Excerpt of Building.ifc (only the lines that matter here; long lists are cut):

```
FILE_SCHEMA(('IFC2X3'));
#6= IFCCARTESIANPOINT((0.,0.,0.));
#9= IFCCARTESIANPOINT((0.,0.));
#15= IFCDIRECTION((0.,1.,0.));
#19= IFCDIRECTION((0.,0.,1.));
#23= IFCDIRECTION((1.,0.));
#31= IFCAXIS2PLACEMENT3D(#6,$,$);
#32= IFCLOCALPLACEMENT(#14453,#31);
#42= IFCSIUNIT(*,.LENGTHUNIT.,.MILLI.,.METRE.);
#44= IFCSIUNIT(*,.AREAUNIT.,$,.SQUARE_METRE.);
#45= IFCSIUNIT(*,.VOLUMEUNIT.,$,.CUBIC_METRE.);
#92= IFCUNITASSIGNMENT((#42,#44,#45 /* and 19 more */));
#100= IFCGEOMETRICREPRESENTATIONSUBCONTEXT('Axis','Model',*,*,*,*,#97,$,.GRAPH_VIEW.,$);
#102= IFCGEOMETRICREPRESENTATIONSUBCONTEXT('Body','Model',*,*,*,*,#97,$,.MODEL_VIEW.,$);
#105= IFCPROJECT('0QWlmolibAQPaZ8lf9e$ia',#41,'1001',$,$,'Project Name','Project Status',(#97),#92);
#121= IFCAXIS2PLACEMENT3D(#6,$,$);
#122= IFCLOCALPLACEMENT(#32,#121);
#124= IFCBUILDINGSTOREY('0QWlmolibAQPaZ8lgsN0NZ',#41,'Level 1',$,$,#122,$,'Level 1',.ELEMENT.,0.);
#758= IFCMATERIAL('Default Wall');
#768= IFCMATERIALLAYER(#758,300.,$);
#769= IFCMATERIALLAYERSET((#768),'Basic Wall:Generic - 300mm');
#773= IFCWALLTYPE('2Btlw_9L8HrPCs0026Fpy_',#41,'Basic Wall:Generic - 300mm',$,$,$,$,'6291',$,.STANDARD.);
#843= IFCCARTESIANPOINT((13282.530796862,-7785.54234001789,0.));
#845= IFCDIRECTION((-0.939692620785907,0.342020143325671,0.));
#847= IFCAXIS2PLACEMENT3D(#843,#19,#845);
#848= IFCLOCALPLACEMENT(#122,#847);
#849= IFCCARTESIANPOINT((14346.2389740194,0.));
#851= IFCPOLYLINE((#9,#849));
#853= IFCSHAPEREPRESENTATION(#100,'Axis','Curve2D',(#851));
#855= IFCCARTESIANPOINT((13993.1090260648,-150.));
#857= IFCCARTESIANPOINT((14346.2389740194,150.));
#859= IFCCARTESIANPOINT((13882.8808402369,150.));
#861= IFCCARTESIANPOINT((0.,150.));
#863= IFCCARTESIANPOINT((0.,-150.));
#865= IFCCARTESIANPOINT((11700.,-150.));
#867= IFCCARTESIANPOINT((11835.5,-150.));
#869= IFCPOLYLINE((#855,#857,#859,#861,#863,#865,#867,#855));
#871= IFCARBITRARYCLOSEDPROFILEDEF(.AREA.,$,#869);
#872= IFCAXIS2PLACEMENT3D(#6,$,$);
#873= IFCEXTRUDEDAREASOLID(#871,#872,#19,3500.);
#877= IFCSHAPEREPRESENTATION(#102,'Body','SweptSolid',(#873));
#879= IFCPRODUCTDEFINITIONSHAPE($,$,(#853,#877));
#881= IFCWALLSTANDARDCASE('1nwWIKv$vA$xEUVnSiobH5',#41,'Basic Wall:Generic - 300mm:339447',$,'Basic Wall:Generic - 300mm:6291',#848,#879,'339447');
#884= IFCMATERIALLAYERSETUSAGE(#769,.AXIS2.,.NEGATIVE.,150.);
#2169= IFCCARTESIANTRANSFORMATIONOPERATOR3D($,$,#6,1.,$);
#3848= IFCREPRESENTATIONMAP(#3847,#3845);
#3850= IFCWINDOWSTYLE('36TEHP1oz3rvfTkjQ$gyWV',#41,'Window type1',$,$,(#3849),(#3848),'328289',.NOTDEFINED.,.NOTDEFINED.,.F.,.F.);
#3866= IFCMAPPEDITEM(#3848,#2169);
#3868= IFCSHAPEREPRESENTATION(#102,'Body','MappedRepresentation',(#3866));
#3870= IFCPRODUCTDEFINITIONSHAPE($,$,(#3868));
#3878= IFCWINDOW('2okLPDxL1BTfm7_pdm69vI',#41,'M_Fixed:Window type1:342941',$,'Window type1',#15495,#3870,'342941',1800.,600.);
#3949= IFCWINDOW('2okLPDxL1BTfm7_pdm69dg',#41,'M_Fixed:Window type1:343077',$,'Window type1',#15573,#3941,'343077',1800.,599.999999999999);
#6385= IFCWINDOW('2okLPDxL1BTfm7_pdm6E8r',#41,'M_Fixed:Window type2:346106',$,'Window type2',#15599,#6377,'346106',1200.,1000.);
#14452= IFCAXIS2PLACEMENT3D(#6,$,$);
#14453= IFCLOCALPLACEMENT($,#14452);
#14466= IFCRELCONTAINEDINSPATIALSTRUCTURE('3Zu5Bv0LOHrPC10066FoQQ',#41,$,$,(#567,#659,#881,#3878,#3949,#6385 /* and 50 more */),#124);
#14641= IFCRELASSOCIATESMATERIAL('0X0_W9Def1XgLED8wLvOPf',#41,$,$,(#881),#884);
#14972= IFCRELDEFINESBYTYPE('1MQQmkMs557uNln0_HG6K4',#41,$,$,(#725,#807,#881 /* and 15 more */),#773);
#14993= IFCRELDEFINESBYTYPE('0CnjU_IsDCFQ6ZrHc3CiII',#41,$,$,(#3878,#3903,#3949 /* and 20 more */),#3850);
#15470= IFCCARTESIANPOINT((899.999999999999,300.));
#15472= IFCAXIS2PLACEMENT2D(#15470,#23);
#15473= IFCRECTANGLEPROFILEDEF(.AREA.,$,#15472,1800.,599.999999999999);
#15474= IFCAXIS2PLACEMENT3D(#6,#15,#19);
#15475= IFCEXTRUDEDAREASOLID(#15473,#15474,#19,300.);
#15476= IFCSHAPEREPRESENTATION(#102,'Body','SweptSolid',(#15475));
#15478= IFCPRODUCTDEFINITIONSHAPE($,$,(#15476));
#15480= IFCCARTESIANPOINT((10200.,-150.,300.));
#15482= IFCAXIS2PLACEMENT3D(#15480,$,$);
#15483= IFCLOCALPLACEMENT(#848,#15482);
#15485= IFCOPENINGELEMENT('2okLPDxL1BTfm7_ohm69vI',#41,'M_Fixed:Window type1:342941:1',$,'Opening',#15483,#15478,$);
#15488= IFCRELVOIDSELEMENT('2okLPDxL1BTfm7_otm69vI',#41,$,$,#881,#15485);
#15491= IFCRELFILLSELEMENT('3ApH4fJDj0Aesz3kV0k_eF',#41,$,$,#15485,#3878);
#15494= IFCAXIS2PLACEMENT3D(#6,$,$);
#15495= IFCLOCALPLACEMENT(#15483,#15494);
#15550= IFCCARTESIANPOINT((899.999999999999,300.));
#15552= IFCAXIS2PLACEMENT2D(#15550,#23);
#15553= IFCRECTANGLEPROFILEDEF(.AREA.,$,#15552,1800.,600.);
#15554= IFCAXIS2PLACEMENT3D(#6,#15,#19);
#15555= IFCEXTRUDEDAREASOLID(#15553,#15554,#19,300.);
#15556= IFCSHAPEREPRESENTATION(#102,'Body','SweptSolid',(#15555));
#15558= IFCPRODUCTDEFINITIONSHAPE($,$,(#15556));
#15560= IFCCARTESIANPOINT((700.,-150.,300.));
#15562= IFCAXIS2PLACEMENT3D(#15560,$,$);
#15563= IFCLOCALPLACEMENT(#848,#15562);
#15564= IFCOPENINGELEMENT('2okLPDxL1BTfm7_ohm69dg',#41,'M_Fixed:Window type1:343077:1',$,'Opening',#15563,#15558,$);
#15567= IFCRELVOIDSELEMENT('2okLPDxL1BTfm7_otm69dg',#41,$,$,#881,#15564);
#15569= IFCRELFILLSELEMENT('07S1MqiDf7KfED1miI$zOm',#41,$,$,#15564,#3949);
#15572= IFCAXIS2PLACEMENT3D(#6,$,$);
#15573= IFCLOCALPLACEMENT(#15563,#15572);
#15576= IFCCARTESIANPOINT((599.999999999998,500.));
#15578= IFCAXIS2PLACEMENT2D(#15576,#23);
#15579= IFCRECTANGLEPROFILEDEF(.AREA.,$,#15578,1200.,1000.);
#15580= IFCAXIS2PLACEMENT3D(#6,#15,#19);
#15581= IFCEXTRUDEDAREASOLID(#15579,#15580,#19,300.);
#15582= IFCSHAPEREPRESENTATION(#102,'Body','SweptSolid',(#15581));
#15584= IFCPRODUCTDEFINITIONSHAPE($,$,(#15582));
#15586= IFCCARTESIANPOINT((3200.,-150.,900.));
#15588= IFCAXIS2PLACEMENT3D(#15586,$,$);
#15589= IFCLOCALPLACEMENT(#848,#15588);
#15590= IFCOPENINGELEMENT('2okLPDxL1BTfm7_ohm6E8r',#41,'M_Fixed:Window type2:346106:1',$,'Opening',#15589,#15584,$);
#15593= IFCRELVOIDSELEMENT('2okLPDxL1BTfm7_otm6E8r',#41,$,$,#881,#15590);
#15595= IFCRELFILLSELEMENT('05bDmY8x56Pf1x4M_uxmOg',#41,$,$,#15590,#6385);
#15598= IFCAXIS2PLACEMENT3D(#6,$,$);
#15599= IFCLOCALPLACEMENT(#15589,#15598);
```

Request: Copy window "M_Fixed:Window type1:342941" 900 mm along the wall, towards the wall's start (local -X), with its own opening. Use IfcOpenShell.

```python
import ifcopenshell
import ifcopenshell.api.feature
import ifcopenshell.api.geometry
import ifcopenshell.api.root
import ifcopenshell.geom
import ifcopenshell.util.element
import ifcopenshell.util.placement
import ifcopenshell.util.shape
import ifcopenshell.util.unit

model = ifcopenshell.open("Building.ifc")
unit_scale = ifcopenshell.util.unit.calculate_unit_scale(model)
settings = ifcopenshell.geom.settings()


def volume(element):
    """Net volume in cubic metres, openings subtracted."""
    shape = ifcopenshell.geom.create_shape(settings, element)
    return ifcopenshell.util.shape.get_volume(shape.geometry)


def reuse_history(source, copy):
    """copy_class also copies each property set's owner history, people and application; keep the originals."""
    for rel in copy.IsDefinedBy:
        if rel.is_a("IfcRelDefinesByProperties") and (history := rel.RelatingPropertyDefinition.OwnerHistory):
            rel.RelatingPropertyDefinition.OwnerHistory = source.OwnerHistory
            ifcopenshell.util.element.remove_deep2(model, history)


window = model.by_id(3878)
opening = window.FillsVoids[0].RelatingOpeningElement
wall = opening.VoidsElements[0].RelatingBuildingElement
before = volume(wall)
shift = ifcopenshell.util.placement.get_local_placement(wall.ObjectPlacement)[:3, 0] * -0.9 / unit_scale

# copy_class copies the void relationship, type, container and properties, but no geometry.
new_opening = ifcopenshell.api.root.copy_class(model, product=opening)
new_opening.Representation = ifcopenshell.util.element.copy_deep(
    model, opening.Representation, exclude=["IfcGeometricRepresentationContext", "IfcRepresentationMap"]
)
new_opening.Name = "M_Fixed:Window type1"
new_window = ifcopenshell.api.root.copy_class(model, product=window)
new_window.Representation = ifcopenshell.util.element.copy_deep(
    model, window.Representation, exclude=["IfcGeometricRepresentationContext", "IfcRepresentationMap"]
)
new_window.Name = "M_Fixed:Window type1"
new_window.Tag = None
reuse_history(window, new_window)
fills = ifcopenshell.api.feature.add_filling(model, opening=new_opening, element=new_window)
fills.OwnerHistory = new_window.OwnerHistory  # required in IFC2X3

for old, new in ((opening, new_opening), (window, new_window)):
    matrix = ifcopenshell.util.placement.get_local_placement(old.ObjectPlacement)
    matrix[:3, 3] += shift
    ifcopenshell.api.geometry.edit_object_placement(model, product=new, matrix=matrix, is_si=False)

after = volume(wall)

print(f"wall volume {before:.3f} -> {after:.3f} m3")

model.write("Building_rev.ifc")
```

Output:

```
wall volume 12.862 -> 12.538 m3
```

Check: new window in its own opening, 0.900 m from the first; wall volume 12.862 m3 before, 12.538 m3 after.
